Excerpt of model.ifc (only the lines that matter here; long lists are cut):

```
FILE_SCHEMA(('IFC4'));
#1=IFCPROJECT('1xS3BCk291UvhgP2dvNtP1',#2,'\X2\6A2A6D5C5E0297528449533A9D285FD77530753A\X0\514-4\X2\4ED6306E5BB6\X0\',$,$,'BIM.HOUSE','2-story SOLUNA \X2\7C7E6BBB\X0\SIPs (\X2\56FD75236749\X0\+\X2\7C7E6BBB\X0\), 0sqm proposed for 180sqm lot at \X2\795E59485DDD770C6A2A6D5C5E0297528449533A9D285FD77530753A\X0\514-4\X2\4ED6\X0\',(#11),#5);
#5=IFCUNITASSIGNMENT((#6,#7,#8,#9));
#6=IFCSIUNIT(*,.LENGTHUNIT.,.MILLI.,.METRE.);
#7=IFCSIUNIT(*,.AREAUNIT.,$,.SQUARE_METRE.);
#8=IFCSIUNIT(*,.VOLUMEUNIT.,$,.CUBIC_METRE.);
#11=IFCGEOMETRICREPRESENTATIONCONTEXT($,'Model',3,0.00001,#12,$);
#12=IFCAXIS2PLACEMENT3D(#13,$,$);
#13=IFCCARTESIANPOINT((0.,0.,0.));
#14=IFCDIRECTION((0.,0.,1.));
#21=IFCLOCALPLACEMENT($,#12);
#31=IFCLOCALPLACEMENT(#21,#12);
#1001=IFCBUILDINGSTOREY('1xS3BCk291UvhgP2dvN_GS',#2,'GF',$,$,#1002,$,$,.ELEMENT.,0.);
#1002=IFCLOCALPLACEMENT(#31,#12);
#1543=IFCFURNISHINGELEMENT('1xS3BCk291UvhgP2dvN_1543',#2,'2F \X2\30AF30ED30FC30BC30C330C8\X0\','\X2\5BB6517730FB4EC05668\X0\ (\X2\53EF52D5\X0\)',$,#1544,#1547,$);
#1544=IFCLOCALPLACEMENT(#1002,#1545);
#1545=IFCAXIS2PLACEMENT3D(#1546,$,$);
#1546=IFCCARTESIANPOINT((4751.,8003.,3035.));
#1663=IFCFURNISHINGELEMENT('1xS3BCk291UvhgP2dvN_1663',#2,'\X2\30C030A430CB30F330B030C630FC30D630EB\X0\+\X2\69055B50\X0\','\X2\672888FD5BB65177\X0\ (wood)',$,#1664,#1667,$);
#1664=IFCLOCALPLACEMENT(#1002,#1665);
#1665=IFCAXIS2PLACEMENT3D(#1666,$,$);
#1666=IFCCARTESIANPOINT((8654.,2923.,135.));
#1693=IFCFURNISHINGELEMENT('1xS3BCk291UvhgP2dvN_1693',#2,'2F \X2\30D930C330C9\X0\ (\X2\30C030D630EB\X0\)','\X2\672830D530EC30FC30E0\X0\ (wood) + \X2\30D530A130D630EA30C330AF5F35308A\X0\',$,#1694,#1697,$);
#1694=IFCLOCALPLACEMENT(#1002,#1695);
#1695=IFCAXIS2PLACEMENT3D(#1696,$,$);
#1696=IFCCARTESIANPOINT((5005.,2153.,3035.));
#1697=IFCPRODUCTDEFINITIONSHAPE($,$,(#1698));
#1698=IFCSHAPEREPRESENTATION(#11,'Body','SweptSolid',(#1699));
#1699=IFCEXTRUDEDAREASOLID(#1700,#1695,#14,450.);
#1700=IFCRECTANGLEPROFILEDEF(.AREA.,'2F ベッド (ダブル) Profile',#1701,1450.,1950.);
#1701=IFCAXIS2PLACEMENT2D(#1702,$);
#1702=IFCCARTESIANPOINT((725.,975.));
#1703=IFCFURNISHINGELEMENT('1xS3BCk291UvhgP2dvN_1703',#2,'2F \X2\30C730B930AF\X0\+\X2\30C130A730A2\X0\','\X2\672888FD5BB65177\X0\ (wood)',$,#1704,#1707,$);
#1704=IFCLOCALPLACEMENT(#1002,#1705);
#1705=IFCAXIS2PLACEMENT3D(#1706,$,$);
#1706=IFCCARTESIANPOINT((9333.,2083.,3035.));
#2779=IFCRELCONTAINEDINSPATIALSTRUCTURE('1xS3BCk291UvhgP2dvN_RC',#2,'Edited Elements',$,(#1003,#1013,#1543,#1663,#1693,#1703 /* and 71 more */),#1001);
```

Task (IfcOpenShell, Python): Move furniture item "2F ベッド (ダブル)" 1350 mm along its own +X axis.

```python
import ifcopenshell
import ifcopenshell.api.geometry
import ifcopenshell.util.placement
import ifcopenshell.util.unit

model = ifcopenshell.open("model.ifc")
unit_scale = ifcopenshell.util.unit.calculate_unit_scale(model)

item = model.by_guid("1xS3BCk291UvhgP2dvN_1693")
matrix = ifcopenshell.util.placement.get_local_placement(item.ObjectPlacement)
matrix[:3, 3] += matrix[:3, 0] * 1.35 / unit_scale
ifcopenshell.api.geometry.edit_object_placement(model, product=item, matrix=matrix, is_si=False)

print(ifcopenshell.util.placement.get_local_placement(item.ObjectPlacement).round(3) + 0.0)

model.write("model_rev.ifc")
```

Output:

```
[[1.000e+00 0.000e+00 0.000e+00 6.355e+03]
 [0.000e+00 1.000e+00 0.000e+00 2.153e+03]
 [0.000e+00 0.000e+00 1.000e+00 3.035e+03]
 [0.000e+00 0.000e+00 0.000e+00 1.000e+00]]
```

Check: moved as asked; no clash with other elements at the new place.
